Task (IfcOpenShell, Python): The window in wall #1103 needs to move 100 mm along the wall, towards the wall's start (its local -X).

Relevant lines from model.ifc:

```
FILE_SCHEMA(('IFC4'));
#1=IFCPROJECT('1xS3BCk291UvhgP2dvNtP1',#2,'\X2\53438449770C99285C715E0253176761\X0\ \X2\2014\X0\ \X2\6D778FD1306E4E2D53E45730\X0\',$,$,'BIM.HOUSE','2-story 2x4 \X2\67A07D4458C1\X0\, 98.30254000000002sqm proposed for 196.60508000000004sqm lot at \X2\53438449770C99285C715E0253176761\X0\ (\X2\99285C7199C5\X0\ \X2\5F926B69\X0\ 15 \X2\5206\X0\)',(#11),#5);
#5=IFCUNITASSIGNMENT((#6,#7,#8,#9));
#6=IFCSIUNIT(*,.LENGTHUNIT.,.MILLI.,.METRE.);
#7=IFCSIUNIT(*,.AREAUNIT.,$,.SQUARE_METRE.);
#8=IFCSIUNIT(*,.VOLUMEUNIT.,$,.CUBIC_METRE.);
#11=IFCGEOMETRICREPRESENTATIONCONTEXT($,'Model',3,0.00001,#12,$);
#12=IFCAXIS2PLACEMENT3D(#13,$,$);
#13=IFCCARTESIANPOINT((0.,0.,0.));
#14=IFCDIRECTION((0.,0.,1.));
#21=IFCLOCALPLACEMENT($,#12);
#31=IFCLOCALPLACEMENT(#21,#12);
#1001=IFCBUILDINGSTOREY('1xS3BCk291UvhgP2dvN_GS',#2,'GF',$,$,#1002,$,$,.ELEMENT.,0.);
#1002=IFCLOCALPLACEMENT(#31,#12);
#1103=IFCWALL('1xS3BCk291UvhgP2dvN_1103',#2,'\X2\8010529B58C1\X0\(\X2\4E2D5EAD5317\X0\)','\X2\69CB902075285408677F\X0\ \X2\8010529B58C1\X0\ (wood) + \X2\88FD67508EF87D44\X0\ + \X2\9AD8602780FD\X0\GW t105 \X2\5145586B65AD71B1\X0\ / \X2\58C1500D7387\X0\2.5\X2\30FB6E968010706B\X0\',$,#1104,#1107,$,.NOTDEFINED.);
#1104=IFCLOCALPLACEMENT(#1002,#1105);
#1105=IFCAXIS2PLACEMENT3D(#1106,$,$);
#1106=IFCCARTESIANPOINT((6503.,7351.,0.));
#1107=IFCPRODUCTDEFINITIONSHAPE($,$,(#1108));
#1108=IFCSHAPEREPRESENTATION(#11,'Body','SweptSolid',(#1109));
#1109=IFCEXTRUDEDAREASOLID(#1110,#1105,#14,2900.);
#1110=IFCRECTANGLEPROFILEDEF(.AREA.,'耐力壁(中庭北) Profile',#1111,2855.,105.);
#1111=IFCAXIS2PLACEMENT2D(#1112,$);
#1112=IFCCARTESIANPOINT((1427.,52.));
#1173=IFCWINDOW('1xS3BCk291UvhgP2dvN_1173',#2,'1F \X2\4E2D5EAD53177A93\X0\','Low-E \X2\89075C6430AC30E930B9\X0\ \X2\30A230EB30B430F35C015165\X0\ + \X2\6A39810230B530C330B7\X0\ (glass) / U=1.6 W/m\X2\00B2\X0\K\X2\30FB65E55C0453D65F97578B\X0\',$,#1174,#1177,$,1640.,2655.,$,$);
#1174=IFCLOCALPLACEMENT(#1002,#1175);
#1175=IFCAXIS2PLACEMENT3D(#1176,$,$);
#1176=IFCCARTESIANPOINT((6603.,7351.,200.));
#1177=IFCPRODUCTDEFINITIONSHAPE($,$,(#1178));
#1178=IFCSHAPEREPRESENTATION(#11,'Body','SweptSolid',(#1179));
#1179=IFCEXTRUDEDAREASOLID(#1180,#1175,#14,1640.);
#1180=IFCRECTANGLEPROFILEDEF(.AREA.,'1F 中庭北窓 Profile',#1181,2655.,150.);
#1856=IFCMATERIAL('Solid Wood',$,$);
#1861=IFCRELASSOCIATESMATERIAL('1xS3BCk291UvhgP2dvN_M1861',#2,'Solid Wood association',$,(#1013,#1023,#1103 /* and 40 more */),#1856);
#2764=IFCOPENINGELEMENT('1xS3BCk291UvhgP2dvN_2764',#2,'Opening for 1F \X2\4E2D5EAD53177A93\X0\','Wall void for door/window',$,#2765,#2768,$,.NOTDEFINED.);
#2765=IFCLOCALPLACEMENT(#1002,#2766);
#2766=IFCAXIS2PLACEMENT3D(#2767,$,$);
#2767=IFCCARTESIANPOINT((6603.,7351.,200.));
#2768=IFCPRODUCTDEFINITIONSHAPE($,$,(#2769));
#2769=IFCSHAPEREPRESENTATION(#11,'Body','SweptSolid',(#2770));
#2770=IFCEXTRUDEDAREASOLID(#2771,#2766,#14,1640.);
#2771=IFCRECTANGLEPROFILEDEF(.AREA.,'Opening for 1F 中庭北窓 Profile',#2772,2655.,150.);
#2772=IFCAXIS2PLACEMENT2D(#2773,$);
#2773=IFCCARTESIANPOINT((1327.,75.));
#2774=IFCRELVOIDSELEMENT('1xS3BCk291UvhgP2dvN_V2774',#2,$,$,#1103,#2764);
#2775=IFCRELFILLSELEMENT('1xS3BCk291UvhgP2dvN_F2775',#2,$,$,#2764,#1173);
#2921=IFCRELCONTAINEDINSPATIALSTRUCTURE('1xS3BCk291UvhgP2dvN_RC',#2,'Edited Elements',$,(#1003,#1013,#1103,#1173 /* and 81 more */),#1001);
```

```python
import ifcopenshell
import ifcopenshell.api.geometry
import ifcopenshell.util.placement
import ifcopenshell.util.unit

model = ifcopenshell.open("model.ifc")
unit_scale = ifcopenshell.util.unit.calculate_unit_scale(model)

window = model.by_guid("1xS3BCk291UvhgP2dvN_1173")
opening = window.FillsVoids[0].RelatingOpeningElement
wall = opening.VoidsElements[0].RelatingBuildingElement

wall_matrix = ifcopenshell.util.placement.get_local_placement(wall.ObjectPlacement)
shift = wall_matrix[:3, 0] * -0.1 / unit_scale
before = ifcopenshell.util.placement.get_local_placement(window.ObjectPlacement)[:3, 3].copy()

# The window is not placed relative to its opening, so move both.
for product in (opening, window):
    matrix = ifcopenshell.util.placement.get_local_placement(product.ObjectPlacement)
    matrix[:3, 3] += shift
    ifcopenshell.api.geometry.edit_object_placement(model, product=product, matrix=matrix, is_si=False)

after = ifcopenshell.util.placement.get_local_placement(window.ObjectPlacement)[:3, 3]
print("window moved by", (after - before).round(3) + 0.0)

model.write("model_updated.ifc")
```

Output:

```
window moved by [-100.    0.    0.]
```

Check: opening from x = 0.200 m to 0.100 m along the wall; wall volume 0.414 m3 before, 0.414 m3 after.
